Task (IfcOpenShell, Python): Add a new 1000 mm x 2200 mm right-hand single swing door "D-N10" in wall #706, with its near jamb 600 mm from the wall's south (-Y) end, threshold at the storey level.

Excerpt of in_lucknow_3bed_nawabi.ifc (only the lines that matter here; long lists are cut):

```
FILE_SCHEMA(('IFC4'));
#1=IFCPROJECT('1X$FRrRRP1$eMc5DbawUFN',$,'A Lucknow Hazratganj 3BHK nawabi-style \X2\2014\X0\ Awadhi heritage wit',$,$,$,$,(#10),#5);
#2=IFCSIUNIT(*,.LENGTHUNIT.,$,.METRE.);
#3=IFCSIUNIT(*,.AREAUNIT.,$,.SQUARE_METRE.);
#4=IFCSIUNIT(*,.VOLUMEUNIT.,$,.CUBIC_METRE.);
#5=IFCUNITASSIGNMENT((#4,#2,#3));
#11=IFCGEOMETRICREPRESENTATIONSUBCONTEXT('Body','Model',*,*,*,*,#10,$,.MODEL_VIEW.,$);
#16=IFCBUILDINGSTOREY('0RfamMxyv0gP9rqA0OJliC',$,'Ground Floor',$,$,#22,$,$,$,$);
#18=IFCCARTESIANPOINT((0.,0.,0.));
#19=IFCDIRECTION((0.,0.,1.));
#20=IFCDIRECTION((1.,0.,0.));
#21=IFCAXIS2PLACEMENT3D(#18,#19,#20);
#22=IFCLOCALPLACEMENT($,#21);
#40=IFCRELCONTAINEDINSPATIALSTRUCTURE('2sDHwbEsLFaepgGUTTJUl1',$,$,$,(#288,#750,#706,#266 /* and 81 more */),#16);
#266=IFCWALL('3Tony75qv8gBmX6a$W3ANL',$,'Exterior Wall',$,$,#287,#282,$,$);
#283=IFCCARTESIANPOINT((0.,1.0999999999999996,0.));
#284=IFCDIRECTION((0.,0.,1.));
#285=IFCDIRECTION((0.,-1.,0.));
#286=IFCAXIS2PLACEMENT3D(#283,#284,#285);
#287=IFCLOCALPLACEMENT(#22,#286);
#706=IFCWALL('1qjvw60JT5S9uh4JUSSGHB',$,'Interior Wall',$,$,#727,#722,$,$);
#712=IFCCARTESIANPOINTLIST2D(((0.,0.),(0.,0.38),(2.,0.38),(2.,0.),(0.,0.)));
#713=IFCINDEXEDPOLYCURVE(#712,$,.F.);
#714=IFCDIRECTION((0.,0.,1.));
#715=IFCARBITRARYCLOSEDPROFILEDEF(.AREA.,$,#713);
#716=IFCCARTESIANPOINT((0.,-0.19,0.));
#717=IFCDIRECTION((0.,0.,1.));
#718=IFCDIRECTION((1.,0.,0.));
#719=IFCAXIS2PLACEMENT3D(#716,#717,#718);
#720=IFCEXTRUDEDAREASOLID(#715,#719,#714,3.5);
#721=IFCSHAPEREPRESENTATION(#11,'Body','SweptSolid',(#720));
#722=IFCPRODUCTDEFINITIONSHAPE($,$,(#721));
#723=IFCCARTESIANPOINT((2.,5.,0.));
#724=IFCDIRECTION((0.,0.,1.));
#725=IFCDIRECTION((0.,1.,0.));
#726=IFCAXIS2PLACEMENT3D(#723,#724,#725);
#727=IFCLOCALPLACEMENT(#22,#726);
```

```python
import numpy as np
import ifcopenshell
import ifcopenshell.api.feature
import ifcopenshell.api.geometry
import ifcopenshell.api.root
import ifcopenshell.api.spatial
import ifcopenshell.geom
import ifcopenshell.util.element
import ifcopenshell.util.placement
import ifcopenshell.util.representation
import ifcopenshell.util.shape
import ifcopenshell.util.unit

model = ifcopenshell.open("in_lucknow_3bed_nawabi.ifc")
unit_scale = ifcopenshell.util.unit.calculate_unit_scale(model)
settings = ifcopenshell.geom.settings()


def volume(element):
    """Net volume in cubic metres, openings subtracted."""
    shape = ifcopenshell.geom.create_shape(settings, element)
    return ifcopenshell.util.shape.get_volume(shape.geometry)


wall = model.by_guid("1qjvw60JT5S9uh4JUSSGHB")
storey = ifcopenshell.util.element.get_container(wall, ifc_class="IfcBuildingStorey")
context = ifcopenshell.util.representation.get_context(model, "Model", "Body", "MODEL_VIEW")
before = volume(wall)

width, height, from_end, sill = 1, 2.2, 0.6, 0.0  # metres

# The wall runs along its own X axis, and the end named is its -X end.
wall_shape = ifcopenshell.geom.create_shape(settings, wall)
x, y, z = ifcopenshell.util.shape.get_vertices(wall_shape.geometry).T
start = x.min() + from_end
face, thickness = float(y.min()), float(y.max() - y.min())
wall_matrix = ifcopenshell.util.placement.get_local_placement(wall.ObjectPlacement)
level = ifcopenshell.util.placement.get_local_placement(storey.ObjectPlacement)[2, 3]


def in_wall(x, y):
    """Placement at x, y metres in the wall's axes, at sill height."""
    matrix = wall_matrix.copy()
    matrix[:, 3] = wall_matrix @ np.array([x / unit_scale, y / unit_scale, 0.0, 1.0])
    matrix[2, 3] = level + sill / unit_scale
    return matrix


# Opening: a box that overshoots both wall faces by 50 mm.
opening = ifcopenshell.api.root.create_entity(model, ifc_class="IfcOpeningElement", predefined_type="OPENING")
box = ifcopenshell.api.geometry.add_wall_representation(
    model, context=context, length=width, height=height, thickness=thickness + 0.1
)
ifcopenshell.api.geometry.assign_representation(model, product=opening, representation=box)
ifcopenshell.api.geometry.edit_object_placement(model, product=opening, matrix=in_wall(start, face - 0.05), is_si=False)
ifcopenshell.api.feature.add_feature(model, feature=opening, element=wall)

door = ifcopenshell.api.root.create_entity(model, ifc_class="IfcDoor", name="D-N10", predefined_type="DOOR")
door.OverallWidth, door.OverallHeight = width / unit_scale, height / unit_scale
door.OperationType = "SINGLE_SWING_RIGHT"
body = ifcopenshell.api.geometry.add_door_representation(
    model,
    context=context,
    overall_width=door.OverallWidth,
    overall_height=door.OverallHeight,
    operation_type="SINGLE_SWING_RIGHT",
    lining_properties={"LiningDepth": thickness / unit_scale, "ThresholdDepth": thickness / unit_scale},
)
ifcopenshell.api.geometry.assign_representation(model, product=door, representation=body)
ifcopenshell.api.spatial.assign_container(model, products=[door], relating_structure=storey)
ifcopenshell.api.feature.add_filling(model, opening=opening, element=door)

# The lining spans the wall, so the door starts at the wall face.
ifcopenshell.api.geometry.edit_object_placement(model, product=door, matrix=in_wall(start, face), is_si=False)

after = volume(wall)

print(f"wall volume {before:.3f} -> {after:.3f} m3")

model.write("in_lucknow_3bed_nawabi_updated.ifc")
```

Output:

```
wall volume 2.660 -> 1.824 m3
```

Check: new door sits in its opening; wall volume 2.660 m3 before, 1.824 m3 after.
